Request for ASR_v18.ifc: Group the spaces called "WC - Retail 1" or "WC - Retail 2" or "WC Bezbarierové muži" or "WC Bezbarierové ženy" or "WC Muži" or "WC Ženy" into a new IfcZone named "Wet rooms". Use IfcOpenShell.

First a look at what the model holds.

```python
import ifcopenshell

model = ifcopenshell.open("ASR_v18.ifc")
print(model.schema)
seen = {}
for space in model.by_type("IfcSpace"):
    seen[space.LongName] = seen.get(space.LongName, 0) + 1
for name, count in sorted(seen.items(), key=str):
    print(count, "x", name)
print("zones:", [z.Name for z in model.by_type("IfcZone")][:20])
```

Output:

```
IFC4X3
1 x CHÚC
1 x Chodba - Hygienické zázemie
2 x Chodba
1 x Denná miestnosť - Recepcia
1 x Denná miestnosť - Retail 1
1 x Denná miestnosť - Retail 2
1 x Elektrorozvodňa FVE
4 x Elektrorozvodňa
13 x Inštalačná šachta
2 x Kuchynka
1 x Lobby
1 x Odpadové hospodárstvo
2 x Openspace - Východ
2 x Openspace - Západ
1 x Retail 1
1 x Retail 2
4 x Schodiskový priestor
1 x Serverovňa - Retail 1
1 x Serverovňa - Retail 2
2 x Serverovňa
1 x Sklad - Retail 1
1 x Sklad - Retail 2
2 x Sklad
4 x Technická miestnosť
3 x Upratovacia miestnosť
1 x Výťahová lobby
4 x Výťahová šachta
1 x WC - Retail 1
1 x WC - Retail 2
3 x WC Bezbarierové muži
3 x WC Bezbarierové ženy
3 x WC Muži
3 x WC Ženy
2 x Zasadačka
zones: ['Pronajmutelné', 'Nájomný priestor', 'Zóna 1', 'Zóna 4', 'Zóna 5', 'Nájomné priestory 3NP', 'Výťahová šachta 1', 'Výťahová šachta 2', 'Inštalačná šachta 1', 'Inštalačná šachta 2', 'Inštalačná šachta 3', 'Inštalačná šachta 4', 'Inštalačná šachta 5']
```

```python
import ifcopenshell
import ifcopenshell.api.group
import ifcopenshell.api.root

model = ifcopenshell.open("ASR_v18.ifc")

names = {"WC - Retail 1", "WC - Retail 2", "WC Bezbarierové muži", "WC Bezbarierové ženy", "WC Muži", "WC Ženy"}
spaces = [s for s in model.by_type("IfcSpace") if s.LongName in names]

zone = ifcopenshell.api.root.create_entity(model, ifc_class="IfcZone", name="Wet rooms")
ifcopenshell.api.group.assign_group(model, products=spaces, group=zone)
print(len(spaces), "spaces in", zone.Name)

model.write("ASR_v18_updated.ifc")
```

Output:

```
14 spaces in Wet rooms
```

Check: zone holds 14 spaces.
